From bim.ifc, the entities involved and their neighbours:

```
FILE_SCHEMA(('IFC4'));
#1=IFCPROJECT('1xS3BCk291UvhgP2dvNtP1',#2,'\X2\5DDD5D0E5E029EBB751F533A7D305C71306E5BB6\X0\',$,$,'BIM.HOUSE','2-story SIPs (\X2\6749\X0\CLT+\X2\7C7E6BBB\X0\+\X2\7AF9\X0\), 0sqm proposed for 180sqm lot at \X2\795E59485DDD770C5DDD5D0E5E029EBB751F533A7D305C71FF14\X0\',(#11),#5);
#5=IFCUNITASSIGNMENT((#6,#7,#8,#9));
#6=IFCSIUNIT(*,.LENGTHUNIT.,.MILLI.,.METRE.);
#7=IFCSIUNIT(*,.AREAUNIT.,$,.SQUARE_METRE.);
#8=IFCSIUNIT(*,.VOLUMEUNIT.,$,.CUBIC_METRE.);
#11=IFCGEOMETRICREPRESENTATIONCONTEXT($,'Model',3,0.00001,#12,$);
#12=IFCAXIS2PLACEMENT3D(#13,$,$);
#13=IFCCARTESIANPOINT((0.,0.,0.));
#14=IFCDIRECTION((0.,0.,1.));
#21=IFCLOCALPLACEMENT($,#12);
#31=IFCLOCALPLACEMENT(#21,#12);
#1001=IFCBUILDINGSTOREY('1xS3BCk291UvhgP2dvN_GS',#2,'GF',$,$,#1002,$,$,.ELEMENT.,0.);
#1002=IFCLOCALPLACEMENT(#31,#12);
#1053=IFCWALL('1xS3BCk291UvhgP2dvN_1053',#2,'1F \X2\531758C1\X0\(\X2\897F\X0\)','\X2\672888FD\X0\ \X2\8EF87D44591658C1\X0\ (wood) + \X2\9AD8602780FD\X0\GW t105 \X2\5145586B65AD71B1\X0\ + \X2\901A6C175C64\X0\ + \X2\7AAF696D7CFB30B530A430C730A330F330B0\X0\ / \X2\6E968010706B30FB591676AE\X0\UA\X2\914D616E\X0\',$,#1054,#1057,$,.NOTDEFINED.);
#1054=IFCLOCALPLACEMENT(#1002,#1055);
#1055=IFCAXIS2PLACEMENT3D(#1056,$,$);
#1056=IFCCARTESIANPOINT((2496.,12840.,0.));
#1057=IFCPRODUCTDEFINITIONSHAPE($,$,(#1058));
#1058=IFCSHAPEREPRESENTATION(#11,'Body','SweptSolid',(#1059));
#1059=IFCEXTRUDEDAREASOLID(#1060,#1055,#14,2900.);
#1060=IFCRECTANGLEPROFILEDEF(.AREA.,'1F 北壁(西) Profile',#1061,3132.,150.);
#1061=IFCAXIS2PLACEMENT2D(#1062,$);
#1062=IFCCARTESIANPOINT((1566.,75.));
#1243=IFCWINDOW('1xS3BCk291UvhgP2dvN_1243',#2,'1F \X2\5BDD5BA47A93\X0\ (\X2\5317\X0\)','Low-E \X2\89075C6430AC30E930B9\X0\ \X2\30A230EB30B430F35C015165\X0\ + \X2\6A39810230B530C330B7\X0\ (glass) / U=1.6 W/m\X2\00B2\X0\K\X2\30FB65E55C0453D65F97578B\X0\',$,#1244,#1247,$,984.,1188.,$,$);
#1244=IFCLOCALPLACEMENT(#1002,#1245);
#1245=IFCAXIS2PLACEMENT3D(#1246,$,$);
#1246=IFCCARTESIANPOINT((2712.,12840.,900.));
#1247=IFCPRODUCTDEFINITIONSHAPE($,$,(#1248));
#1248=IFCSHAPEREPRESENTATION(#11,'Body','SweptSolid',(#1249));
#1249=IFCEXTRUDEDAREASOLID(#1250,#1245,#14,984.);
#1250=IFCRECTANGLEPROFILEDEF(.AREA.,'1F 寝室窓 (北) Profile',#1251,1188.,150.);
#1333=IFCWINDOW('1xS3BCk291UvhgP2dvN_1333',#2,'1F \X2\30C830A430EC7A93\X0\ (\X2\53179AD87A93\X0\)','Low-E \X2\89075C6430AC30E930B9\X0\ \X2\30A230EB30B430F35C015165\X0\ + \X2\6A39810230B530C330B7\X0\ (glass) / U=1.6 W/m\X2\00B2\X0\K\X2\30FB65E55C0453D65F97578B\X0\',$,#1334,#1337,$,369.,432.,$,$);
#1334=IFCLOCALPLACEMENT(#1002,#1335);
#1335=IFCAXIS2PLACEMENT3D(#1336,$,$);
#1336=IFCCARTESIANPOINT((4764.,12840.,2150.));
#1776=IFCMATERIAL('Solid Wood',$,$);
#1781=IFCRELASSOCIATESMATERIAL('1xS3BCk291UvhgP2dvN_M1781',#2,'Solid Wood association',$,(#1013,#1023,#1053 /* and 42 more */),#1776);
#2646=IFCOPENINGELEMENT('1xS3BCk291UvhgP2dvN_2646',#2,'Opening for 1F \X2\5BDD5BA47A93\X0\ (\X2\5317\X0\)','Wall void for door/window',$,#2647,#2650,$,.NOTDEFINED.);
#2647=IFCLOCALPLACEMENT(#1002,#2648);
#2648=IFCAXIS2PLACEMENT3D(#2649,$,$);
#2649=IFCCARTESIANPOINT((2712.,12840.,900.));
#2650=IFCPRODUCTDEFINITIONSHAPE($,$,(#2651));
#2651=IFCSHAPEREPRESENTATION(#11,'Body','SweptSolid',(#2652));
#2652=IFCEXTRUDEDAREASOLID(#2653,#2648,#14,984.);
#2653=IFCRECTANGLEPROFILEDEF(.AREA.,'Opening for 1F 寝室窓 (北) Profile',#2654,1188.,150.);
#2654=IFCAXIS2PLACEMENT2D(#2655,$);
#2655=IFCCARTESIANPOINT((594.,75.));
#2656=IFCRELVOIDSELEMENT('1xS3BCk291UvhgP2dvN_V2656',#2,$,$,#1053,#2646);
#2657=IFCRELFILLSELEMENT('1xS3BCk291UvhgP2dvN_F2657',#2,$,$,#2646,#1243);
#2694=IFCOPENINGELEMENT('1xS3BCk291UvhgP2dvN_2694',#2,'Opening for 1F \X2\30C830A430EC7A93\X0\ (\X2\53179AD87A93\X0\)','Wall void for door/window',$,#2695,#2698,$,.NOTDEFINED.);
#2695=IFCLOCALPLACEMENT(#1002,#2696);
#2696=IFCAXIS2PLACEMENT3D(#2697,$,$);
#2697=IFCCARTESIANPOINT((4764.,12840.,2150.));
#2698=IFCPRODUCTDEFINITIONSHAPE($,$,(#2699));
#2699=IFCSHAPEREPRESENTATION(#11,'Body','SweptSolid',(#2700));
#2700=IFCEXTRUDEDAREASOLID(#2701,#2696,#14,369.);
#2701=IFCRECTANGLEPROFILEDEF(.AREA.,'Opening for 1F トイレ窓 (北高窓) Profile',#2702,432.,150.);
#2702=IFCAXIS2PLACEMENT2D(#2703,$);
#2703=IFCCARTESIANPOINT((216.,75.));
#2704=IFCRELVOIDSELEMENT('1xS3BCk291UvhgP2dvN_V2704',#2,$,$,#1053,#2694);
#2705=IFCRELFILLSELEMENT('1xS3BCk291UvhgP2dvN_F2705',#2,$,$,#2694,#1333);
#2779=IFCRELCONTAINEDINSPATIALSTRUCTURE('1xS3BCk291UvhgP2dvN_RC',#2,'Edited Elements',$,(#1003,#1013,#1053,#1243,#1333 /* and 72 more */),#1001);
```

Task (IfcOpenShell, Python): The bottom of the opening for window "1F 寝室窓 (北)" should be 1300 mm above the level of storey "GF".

```python
import numpy as np
import ifcopenshell
import ifcopenshell.api.geometry
import ifcopenshell.geom
import ifcopenshell.util.element
import ifcopenshell.util.placement
import ifcopenshell.util.shape
import ifcopenshell.util.unit

model = ifcopenshell.open("bim.ifc")
unit_scale = ifcopenshell.util.unit.calculate_unit_scale(model)

window = model.by_id(1243)
opening = window.FillsVoids[0].RelatingOpeningElement
storey = ifcopenshell.util.element.get_container(window, ifc_class="IfcBuildingStorey")
level = ifcopenshell.util.placement.get_local_placement(storey.ObjectPlacement)[2, 3]

# The opening's origin need not be at the sill, so measure its lowest point.
shape = ifcopenshell.geom.create_shape(ifcopenshell.geom.settings(), opening)
bottom = ifcopenshell.util.shape.get_shape_bottom_elevation(shape, shape.geometry) / unit_scale
dz = level + 1.3 / unit_scale - bottom

shift = np.array([0.0, 0.0, dz])
# The window is not placed relative to its opening, so move both.
for product in (opening, window):
    matrix = ifcopenshell.util.placement.get_local_placement(product.ObjectPlacement)
    matrix[:3, 3] += shift
    ifcopenshell.api.geometry.edit_object_placement(model, product=product, matrix=matrix, is_si=False)

print(f"moved by {dz * unit_scale:+.3f} m")

model.write("bim_edited.ifc")
```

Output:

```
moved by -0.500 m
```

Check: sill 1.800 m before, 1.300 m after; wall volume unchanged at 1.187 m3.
